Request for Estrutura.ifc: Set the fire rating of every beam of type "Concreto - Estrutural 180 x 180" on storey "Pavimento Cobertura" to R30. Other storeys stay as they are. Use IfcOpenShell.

First a look at what the model holds.

```python
import ifcopenshell
import ifcopenshell.util.element

model = ifcopenshell.open("Estrutura.ifc")
print(model.schema)
storey = next(s for s in model.by_type("IfcBuildingStorey") if s.Name == "Pavimento Cobertura")
beams = [e for e in ifcopenshell.util.element.get_decomposition(storey) if e.is_a("IfcBeam")]
seen = {}
for e in beams:
    element_type = ifcopenshell.util.element.get_type(e)
    key = (element_type.Name if element_type != e and element_type else None, ifcopenshell.util.element.get_pset(e, "Pset_BeamCommon", "FireRating"))
    seen[key] = seen.get(key, 0) + 1
for (name, value), count in sorted(seen.items(), key=str):
    print(count, "x", name, "|", value)
```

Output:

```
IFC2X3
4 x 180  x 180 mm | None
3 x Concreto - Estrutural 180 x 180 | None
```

```python
import ifcopenshell
import ifcopenshell.api.pset
import ifcopenshell.util.element

model = ifcopenshell.open("Estrutura.ifc")

storey = next(s for s in model.by_type("IfcBuildingStorey") if s.Name == "Pavimento Cobertura")
beams = [e for e in ifcopenshell.util.element.get_decomposition(storey) if e.is_a("IfcBeam")]

count = 0
for e in beams:
    element_type = ifcopenshell.util.element.get_type(e)
    if element_type in (None, e) or element_type.Name != "Concreto - Estrutural 180 x 180":
        continue
    # add_pset returns the element's existing set when there is one.
    pset = ifcopenshell.api.pset.add_pset(model, product=e, name="Pset_BeamCommon")
    ifcopenshell.api.pset.edit_pset(model, pset=pset, properties={"FireRating": "R30"})
    count += 1

print(count, "beams updated")

model.write("Estrutura_updated.ifc")
```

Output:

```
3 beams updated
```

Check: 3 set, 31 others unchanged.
